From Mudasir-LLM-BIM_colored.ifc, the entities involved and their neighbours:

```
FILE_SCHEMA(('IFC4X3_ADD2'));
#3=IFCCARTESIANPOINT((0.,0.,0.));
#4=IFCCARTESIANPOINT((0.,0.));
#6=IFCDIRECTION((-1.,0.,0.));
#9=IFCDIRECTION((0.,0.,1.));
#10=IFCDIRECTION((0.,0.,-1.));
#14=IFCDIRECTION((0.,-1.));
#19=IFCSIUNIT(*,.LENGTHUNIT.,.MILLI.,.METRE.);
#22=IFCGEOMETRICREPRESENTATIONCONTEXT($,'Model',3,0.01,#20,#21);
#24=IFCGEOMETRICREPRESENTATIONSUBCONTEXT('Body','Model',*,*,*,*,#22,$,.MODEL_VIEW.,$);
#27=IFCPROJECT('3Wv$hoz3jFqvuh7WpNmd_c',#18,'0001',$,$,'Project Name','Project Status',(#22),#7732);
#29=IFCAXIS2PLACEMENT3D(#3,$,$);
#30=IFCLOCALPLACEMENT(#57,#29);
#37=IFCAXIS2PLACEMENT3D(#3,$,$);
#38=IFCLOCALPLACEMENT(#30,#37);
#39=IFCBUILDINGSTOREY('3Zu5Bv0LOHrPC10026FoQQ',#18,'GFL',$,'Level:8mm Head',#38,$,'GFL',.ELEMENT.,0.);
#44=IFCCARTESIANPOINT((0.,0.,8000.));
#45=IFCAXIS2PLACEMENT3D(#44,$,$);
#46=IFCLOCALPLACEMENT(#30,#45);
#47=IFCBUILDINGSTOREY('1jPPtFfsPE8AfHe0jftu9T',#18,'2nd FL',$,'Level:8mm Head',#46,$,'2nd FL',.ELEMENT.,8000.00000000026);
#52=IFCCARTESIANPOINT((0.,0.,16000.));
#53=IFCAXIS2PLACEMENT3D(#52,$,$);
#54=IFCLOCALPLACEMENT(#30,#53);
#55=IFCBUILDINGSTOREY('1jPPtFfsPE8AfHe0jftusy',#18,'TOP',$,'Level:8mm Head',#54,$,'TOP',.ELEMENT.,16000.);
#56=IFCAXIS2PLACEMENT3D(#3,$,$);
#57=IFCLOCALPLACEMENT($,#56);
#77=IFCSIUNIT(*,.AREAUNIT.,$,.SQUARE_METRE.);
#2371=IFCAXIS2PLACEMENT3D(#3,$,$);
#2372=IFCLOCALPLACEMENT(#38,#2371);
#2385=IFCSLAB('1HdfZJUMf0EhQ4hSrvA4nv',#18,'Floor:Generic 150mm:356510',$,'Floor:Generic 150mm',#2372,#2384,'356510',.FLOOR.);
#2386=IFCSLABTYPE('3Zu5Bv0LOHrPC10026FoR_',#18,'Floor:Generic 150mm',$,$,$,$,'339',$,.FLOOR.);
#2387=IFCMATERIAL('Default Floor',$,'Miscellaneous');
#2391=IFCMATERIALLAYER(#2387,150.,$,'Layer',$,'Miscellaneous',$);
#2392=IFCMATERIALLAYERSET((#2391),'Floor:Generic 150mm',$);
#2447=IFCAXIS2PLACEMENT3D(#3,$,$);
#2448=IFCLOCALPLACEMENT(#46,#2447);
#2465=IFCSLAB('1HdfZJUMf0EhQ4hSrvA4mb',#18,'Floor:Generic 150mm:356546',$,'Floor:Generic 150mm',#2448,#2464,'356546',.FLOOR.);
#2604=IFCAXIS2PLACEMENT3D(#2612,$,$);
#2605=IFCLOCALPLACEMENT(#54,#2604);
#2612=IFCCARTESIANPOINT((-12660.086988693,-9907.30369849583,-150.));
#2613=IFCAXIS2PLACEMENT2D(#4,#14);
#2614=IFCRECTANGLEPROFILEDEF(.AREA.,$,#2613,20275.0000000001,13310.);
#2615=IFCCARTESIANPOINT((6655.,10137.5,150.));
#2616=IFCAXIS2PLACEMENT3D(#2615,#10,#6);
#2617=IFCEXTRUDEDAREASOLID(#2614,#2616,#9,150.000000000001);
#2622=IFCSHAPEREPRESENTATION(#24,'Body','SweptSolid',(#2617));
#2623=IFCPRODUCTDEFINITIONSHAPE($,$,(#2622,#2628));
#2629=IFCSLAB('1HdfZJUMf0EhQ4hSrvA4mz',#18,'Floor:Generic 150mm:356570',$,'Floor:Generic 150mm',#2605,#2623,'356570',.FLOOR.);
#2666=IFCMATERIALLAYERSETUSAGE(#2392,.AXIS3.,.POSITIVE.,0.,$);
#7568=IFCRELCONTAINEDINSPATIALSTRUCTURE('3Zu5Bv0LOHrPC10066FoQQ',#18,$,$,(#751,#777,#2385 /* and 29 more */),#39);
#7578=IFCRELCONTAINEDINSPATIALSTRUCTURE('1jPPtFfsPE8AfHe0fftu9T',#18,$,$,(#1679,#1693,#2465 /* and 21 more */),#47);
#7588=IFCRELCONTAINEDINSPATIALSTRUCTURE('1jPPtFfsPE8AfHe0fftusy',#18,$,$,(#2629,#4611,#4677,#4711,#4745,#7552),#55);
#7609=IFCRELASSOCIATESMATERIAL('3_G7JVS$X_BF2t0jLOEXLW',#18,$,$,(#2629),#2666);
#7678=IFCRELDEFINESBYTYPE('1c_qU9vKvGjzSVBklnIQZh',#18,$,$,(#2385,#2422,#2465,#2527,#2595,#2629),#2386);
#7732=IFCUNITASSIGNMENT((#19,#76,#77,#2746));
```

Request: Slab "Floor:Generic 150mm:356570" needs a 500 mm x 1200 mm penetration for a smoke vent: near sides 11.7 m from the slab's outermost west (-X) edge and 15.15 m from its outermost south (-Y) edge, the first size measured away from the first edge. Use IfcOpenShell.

```python
import numpy as np
import ifcopenshell
import ifcopenshell.api.feature
import ifcopenshell.api.geometry
import ifcopenshell.api.root
import ifcopenshell.geom
import ifcopenshell.util.placement
import ifcopenshell.util.representation
import ifcopenshell.util.shape
import ifcopenshell.util.unit

model = ifcopenshell.open("Mudasir-LLM-BIM_colored.ifc")
unit_scale = ifcopenshell.util.unit.calculate_unit_scale(model)
settings = ifcopenshell.geom.settings()


def volume(element):
    """Net volume in cubic metres, openings subtracted."""
    shape = ifcopenshell.geom.create_shape(settings, element)
    return ifcopenshell.util.shape.get_volume(shape.geometry)


slab = model.by_id(2629)
before = volume(slab)

# Extent in the slab's own axes, in metres. The edges named are its -X and -Y sides.
slab_shape = ifcopenshell.geom.create_shape(settings, slab)
vertices = ifcopenshell.util.shape.get_vertices(slab_shape.geometry)
x_min, y_min, bottom = vertices.min(axis=0)
top = vertices[:, 2].max()

opening = ifcopenshell.api.root.create_entity(model, ifc_class="IfcOpeningElement", name="Smoke vent opening", predefined_type="OPENING")
context = ifcopenshell.util.representation.get_context(model, "Model", "Body", "MODEL_VIEW")
width, depth = 0.5, 1.2
outline = [(0.0, 0.0), (width, 0.0), (width, depth), (0.0, depth), (0.0, 0.0)]
# Overshoot both faces by 50 mm so the cut is clean.
shape = ifcopenshell.api.geometry.add_slab_representation(
    model, context=context, depth=top - bottom + 0.1, polyline=outline
)
ifcopenshell.api.geometry.assign_representation(model, product=opening, representation=shape)

matrix = ifcopenshell.util.placement.get_local_placement(slab.ObjectPlacement)
matrix[:, 3] = matrix @ np.append(np.array([x_min + 11.7, y_min + 15.15, bottom - 0.05]) / unit_scale, 1.0)
ifcopenshell.api.geometry.edit_object_placement(model, product=opening, matrix=matrix, is_si=False)
ifcopenshell.api.feature.add_feature(model, feature=opening, element=slab)

after = volume(slab)

print(f"slab volume {before:.3f} -> {after:.3f} m3")

model.write("Mudasir-LLM-BIM_colored_edited.ifc")
```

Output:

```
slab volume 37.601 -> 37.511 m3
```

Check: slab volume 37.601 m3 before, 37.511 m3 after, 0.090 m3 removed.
